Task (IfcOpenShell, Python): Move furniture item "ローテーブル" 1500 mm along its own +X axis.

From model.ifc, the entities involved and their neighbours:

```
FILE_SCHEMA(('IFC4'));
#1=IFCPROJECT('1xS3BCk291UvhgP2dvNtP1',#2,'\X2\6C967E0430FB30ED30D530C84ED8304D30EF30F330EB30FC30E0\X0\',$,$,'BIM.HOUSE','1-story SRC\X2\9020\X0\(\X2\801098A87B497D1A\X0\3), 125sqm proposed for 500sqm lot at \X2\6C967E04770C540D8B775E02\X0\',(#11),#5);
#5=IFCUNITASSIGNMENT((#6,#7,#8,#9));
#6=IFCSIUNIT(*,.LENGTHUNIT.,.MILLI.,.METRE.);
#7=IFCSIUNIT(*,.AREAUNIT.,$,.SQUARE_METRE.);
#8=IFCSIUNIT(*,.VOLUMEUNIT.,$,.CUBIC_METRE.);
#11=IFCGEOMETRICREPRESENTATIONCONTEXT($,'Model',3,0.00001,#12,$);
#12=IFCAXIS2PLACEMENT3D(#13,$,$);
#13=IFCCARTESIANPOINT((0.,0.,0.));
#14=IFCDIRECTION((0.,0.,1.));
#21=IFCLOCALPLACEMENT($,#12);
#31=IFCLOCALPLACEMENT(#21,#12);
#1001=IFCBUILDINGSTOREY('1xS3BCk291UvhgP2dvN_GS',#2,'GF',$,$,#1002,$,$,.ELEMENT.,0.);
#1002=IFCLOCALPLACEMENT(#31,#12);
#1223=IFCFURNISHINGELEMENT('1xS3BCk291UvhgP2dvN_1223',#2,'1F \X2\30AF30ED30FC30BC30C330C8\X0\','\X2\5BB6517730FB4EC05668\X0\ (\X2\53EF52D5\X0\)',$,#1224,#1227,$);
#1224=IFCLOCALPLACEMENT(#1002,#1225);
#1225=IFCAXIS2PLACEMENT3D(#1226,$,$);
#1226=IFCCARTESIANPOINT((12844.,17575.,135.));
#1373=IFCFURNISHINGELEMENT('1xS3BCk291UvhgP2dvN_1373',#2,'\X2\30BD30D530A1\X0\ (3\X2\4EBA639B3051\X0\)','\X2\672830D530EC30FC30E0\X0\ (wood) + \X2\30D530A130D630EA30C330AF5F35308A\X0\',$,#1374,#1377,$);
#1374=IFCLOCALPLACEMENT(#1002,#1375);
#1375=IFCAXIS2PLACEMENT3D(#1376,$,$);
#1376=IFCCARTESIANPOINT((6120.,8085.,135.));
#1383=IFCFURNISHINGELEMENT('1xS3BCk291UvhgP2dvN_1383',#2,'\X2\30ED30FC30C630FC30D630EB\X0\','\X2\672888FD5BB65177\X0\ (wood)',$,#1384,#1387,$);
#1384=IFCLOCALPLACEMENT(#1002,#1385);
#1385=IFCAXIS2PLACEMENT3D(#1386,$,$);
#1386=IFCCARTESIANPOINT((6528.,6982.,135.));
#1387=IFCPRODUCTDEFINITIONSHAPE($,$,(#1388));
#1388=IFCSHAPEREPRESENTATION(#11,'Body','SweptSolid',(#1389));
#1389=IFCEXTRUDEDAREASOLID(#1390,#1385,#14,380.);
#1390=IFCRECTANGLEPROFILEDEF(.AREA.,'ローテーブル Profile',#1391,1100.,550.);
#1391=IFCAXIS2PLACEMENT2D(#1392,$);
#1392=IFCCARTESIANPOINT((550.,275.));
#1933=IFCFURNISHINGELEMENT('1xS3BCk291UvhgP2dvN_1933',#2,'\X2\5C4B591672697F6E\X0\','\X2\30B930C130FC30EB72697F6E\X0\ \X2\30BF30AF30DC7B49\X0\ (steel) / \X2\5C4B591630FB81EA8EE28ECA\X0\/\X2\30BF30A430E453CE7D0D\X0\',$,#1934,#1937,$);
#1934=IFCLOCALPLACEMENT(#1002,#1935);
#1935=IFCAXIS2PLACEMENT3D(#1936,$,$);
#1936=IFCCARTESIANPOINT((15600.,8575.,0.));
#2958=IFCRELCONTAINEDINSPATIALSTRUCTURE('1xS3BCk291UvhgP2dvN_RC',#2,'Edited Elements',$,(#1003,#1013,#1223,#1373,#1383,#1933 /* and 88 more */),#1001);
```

```python
import ifcopenshell
import ifcopenshell.api.geometry
import ifcopenshell.util.placement

model = ifcopenshell.open("model.ifc")

item = model.by_guid("1xS3BCk291UvhgP2dvN_1383")
matrix = ifcopenshell.util.placement.get_local_placement(item.ObjectPlacement)
matrix[:3, 3] += matrix[:3, 0] * 1500.0
ifcopenshell.api.geometry.edit_object_placement(model, product=item, matrix=matrix, is_si=False)

print(ifcopenshell.util.placement.get_local_placement(item.ObjectPlacement).round(3) + 0.0)

model.write("model_v2.ifc")
```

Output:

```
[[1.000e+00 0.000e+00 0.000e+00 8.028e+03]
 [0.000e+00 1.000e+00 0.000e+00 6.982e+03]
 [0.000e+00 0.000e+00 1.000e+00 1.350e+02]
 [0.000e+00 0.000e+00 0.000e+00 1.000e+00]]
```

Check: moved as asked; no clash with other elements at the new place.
